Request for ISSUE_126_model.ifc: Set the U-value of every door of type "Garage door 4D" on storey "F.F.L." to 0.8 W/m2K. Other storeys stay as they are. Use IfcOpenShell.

First a look at what the model holds.

```python
import ifcopenshell
import ifcopenshell.util.element

model = ifcopenshell.open("ISSUE_126_model.ifc")
print(model.schema)
storey = next(s for s in model.by_type("IfcBuildingStorey") if s.Name == "F.F.L.")
doors = [e for e in ifcopenshell.util.element.get_decomposition(storey) if e.is_a("IfcDoor")]
seen = {}
for e in doors:
    element_type = ifcopenshell.util.element.get_type(e)
    key = (element_type.Name if element_type != e and element_type else None, ifcopenshell.util.element.get_pset(e, "Pset_DoorCommon", "ThermalTransmittance"))
    seen[key] = seen.get(key, 0) + 1
for (name, value), count in sorted(seen.items(), key=str):
    print(count, "x", name, "|", value)
```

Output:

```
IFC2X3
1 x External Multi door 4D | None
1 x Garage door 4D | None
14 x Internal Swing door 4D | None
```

```python
import ifcopenshell
import ifcopenshell.api.pset
import ifcopenshell.util.element

model = ifcopenshell.open("ISSUE_126_model.ifc")

storey = next(s for s in model.by_type("IfcBuildingStorey") if s.Name == "F.F.L.")
doors = [e for e in ifcopenshell.util.element.get_decomposition(storey) if e.is_a("IfcDoor")]

count = 0
for e in doors:
    element_type = ifcopenshell.util.element.get_type(e)
    if element_type in (None, e) or element_type.Name != "Garage door 4D":
        continue
    # add_pset returns the element's existing set when there is one.
    pset = ifcopenshell.api.pset.add_pset(model, product=e, name="Pset_DoorCommon")
    ifcopenshell.api.pset.edit_pset(model, pset=pset, properties={"ThermalTransmittance": 0.8})
    count += 1

print(count, "doors updated")

model.write("ISSUE_126_model_v2.ifc")
```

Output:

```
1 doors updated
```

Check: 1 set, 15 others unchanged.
